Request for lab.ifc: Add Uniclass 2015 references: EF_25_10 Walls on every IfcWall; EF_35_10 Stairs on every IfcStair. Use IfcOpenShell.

First a look at what the model holds.

```python
import ifcopenshell

model = ifcopenshell.open("lab.ifc")
print(model.schema)
print("classifications:", [c.Name for c in model.by_type("IfcClassification")])
for ifc_class in ("IfcDoor", "IfcRoof", "IfcStair", "IfcWall", "IfcWindow"):
    print(ifc_class, len(model.by_type(ifc_class)))
```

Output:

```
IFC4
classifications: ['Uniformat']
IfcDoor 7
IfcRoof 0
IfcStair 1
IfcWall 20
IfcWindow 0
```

```python
import ifcopenshell
import ifcopenshell.api.classification

model = ifcopenshell.open("lab.ifc")

system = ifcopenshell.api.classification.add_classification(model, classification="Uniclass 2015")

codes = {
    "IfcWall": ("EF_25_10", "Walls"),
    "IfcStair": ("EF_35_10", "Stairs"),
}
for ifc_class, (code, name) in codes.items():
    products = model.by_type(ifc_class)
    ifcopenshell.api.classification.add_reference(
        model, products=products, classification=system, identification=code, name=name
    )
    print(code, len(products))

model.write("lab-out.ifc")
```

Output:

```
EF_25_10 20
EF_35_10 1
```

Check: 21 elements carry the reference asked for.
